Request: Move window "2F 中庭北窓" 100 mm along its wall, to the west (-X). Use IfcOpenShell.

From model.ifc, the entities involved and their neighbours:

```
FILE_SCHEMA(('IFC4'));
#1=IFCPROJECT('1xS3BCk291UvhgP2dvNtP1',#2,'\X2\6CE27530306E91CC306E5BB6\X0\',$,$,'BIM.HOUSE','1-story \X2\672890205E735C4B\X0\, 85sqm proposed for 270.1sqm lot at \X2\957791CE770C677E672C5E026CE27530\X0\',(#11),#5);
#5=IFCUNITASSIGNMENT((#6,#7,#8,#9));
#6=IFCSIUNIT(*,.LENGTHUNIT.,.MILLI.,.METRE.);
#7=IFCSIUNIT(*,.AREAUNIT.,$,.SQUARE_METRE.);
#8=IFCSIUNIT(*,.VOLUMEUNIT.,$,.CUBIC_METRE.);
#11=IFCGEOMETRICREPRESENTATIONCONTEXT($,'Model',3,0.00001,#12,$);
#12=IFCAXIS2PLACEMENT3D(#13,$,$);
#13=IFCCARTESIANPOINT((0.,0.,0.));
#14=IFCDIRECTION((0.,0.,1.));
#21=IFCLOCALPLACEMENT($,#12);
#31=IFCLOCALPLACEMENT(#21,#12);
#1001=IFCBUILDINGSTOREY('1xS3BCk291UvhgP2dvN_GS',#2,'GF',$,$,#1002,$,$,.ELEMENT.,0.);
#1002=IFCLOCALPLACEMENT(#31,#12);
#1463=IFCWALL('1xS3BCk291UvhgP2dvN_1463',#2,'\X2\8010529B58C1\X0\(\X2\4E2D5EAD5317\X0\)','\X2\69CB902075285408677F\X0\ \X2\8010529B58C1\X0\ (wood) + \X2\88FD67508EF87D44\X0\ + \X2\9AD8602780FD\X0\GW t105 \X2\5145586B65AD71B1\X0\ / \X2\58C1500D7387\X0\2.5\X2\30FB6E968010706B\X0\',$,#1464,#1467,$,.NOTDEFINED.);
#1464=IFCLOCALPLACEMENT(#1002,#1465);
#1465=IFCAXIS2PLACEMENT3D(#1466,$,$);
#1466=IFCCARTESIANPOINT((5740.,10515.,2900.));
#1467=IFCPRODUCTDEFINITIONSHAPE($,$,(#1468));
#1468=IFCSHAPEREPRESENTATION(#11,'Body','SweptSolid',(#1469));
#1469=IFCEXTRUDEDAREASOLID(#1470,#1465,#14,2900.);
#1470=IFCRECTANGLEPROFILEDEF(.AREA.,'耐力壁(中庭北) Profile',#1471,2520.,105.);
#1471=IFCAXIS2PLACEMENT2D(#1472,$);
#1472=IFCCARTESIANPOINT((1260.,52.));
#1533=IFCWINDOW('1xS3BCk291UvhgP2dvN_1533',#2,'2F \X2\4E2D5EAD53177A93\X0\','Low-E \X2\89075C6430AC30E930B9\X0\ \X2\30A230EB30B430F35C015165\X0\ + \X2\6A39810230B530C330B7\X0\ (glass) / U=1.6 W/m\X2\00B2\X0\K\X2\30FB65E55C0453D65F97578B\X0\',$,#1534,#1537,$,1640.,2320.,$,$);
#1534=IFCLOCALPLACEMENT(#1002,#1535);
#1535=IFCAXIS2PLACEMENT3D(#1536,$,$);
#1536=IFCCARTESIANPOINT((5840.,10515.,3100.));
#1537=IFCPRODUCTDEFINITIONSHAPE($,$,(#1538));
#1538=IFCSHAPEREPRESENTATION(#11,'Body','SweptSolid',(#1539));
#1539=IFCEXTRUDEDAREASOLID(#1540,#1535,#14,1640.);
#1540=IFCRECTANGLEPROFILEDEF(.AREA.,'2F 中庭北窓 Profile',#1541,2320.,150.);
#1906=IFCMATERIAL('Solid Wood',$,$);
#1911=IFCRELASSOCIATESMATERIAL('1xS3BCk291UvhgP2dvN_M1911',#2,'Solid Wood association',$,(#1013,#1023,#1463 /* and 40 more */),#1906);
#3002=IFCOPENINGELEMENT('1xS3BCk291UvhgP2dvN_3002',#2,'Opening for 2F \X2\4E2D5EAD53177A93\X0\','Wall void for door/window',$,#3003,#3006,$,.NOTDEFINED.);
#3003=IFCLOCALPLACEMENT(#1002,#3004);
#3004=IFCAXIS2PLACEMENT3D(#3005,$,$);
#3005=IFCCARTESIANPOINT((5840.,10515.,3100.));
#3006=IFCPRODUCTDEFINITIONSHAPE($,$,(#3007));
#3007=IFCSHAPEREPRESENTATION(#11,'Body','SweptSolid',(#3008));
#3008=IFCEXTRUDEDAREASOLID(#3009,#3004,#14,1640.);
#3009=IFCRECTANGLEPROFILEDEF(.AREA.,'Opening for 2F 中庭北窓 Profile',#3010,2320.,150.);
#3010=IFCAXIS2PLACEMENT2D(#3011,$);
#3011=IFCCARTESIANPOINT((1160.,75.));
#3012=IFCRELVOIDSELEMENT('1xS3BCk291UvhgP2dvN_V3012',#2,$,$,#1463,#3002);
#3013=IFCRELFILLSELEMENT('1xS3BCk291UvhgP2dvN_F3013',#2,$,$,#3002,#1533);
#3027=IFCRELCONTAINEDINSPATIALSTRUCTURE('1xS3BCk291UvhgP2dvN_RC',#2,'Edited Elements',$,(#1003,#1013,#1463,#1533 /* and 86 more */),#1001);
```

```python
import ifcopenshell
import ifcopenshell.api.geometry
import ifcopenshell.util.placement

model = ifcopenshell.open("model.ifc")

window = model.by_guid("1xS3BCk291UvhgP2dvN_1533")
opening = window.FillsVoids[0].RelatingOpeningElement
wall = opening.VoidsElements[0].RelatingBuildingElement

wall_matrix = ifcopenshell.util.placement.get_local_placement(wall.ObjectPlacement)
shift = wall_matrix[:3, 0] * -100.0
before = ifcopenshell.util.placement.get_local_placement(window.ObjectPlacement)[:3, 3].copy()

# The window is not placed relative to its opening, so move both.
for product in (opening, window):
    matrix = ifcopenshell.util.placement.get_local_placement(product.ObjectPlacement)
    matrix[:3, 3] += shift
    ifcopenshell.api.geometry.edit_object_placement(model, product=product, matrix=matrix, is_si=False)

after = ifcopenshell.util.placement.get_local_placement(window.ObjectPlacement)[:3, 3]
print("window moved by", (after - before).round(3) + 0.0)

model.write("model-out.ifc")
```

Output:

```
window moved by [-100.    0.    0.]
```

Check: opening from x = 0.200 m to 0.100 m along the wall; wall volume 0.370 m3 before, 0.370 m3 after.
